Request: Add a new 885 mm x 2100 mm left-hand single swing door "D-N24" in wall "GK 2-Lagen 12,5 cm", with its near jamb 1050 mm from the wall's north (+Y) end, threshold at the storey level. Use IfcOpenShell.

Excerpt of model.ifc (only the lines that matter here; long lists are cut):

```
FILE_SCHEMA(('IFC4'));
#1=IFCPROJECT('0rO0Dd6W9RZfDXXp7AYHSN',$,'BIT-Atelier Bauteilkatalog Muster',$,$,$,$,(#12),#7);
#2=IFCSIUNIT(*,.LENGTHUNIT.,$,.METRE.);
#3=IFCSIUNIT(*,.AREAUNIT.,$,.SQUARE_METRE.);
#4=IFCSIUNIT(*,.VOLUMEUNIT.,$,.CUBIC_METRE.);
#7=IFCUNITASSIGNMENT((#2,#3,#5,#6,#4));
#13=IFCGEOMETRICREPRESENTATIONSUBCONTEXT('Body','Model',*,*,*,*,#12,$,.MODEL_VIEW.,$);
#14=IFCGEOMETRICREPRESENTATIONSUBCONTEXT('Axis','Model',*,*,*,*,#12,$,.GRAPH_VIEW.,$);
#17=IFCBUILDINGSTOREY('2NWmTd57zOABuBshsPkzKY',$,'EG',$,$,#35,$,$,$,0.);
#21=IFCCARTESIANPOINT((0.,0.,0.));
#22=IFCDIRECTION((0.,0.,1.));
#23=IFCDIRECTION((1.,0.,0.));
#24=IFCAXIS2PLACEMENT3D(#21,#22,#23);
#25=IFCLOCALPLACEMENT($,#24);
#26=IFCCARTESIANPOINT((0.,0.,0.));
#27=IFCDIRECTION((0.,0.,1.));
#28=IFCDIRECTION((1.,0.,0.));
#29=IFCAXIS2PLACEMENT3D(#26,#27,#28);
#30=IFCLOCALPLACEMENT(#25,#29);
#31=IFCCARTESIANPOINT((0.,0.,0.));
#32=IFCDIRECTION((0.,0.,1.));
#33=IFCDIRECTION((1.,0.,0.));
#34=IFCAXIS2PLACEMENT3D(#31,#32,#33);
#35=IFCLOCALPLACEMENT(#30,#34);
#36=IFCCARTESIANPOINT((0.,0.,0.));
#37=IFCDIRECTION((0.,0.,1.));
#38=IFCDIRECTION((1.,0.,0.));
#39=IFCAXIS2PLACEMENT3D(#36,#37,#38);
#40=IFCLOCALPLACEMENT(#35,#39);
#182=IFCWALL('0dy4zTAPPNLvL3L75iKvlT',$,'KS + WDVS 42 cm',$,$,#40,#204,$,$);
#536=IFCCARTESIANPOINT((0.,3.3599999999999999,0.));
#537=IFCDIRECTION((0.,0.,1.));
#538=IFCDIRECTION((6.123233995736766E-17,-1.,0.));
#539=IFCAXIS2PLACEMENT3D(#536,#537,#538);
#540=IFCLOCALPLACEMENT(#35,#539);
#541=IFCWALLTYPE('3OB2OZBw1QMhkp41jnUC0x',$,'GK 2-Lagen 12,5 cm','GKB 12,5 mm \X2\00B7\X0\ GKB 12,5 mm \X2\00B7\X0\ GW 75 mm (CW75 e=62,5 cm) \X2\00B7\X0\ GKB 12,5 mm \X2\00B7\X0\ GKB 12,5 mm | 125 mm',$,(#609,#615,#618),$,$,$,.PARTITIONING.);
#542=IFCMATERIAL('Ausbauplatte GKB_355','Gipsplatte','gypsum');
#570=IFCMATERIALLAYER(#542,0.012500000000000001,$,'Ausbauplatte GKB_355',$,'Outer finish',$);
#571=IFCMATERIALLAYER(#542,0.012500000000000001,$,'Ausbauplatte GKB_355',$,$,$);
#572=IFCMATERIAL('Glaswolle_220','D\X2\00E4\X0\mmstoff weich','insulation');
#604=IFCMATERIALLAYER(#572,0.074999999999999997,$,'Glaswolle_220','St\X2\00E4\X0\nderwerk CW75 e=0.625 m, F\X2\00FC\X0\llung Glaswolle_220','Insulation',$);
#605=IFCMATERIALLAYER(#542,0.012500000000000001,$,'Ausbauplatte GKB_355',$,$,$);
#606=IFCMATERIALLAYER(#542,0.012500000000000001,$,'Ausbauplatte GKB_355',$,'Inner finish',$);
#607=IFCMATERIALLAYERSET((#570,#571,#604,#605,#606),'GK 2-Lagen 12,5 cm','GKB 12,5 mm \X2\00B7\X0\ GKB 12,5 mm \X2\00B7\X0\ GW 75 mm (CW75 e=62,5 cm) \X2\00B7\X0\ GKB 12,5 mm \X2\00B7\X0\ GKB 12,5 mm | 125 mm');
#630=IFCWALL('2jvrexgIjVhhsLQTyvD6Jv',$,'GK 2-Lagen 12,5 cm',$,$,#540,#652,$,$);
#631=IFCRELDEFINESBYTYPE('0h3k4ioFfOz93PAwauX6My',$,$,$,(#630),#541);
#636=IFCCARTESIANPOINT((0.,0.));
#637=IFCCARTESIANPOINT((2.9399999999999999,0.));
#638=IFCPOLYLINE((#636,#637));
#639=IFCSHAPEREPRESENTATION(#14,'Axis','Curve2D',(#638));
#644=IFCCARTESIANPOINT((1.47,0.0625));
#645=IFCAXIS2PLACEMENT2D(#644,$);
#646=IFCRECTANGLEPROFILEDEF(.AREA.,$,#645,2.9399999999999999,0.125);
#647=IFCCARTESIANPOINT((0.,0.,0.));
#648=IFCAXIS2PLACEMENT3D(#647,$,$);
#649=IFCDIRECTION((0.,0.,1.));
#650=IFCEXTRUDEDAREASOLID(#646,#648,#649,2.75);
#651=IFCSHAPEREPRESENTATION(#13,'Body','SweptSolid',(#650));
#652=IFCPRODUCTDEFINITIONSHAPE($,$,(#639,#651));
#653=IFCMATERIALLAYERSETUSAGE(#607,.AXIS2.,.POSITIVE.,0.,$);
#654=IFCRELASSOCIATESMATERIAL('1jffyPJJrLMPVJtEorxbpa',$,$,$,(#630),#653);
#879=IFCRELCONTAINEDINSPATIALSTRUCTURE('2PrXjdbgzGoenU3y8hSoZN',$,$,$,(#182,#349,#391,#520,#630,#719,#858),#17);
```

```python
import numpy as np
import ifcopenshell
import ifcopenshell.api.feature
import ifcopenshell.api.geometry
import ifcopenshell.api.root
import ifcopenshell.api.spatial
import ifcopenshell.geom
import ifcopenshell.util.element
import ifcopenshell.util.placement
import ifcopenshell.util.representation
import ifcopenshell.util.shape
import ifcopenshell.util.unit

model = ifcopenshell.open("model.ifc")
unit_scale = ifcopenshell.util.unit.calculate_unit_scale(model)
settings = ifcopenshell.geom.settings()


def volume(element):
    """Net volume in cubic metres, openings subtracted."""
    shape = ifcopenshell.geom.create_shape(settings, element)
    return ifcopenshell.util.shape.get_volume(shape.geometry)


wall = model.by_guid("2jvrexgIjVhhsLQTyvD6Jv")
storey = ifcopenshell.util.element.get_container(wall, ifc_class="IfcBuildingStorey")
context = ifcopenshell.util.representation.get_context(model, "Model", "Body", "MODEL_VIEW")
before = volume(wall)

width, height, from_end, sill = 0.885, 2.1, 1.05, 0.0  # metres

# The wall runs along its own X axis, and the end named is its -X end.
wall_shape = ifcopenshell.geom.create_shape(settings, wall)
x, y, z = ifcopenshell.util.shape.get_vertices(wall_shape.geometry).T
start = x.min() + from_end
face, thickness = float(y.min()), float(y.max() - y.min())
wall_matrix = ifcopenshell.util.placement.get_local_placement(wall.ObjectPlacement)
level = ifcopenshell.util.placement.get_local_placement(storey.ObjectPlacement)[2, 3]


def in_wall(x, y):
    """Placement at x, y metres in the wall's axes, at sill height."""
    matrix = wall_matrix.copy()
    matrix[:, 3] = wall_matrix @ np.array([x / unit_scale, y / unit_scale, 0.0, 1.0])
    matrix[2, 3] = level + sill / unit_scale
    return matrix


# Opening: a box that overshoots both wall faces by 50 mm.
opening = ifcopenshell.api.root.create_entity(model, ifc_class="IfcOpeningElement", predefined_type="OPENING")
box = ifcopenshell.api.geometry.add_wall_representation(
    model, context=context, length=width, height=height, thickness=thickness + 0.1
)
ifcopenshell.api.geometry.assign_representation(model, product=opening, representation=box)
ifcopenshell.api.geometry.edit_object_placement(model, product=opening, matrix=in_wall(start, face - 0.05), is_si=False)
ifcopenshell.api.feature.add_feature(model, feature=opening, element=wall)

door = ifcopenshell.api.root.create_entity(model, ifc_class="IfcDoor", name="D-N24", predefined_type="DOOR")
door.OverallWidth, door.OverallHeight = width / unit_scale, height / unit_scale
door.OperationType = "SINGLE_SWING_LEFT"
body = ifcopenshell.api.geometry.add_door_representation(
    model,
    context=context,
    overall_width=door.OverallWidth,
    overall_height=door.OverallHeight,
    operation_type="SINGLE_SWING_LEFT",
    lining_properties={"LiningDepth": thickness / unit_scale, "ThresholdDepth": thickness / unit_scale},
)
ifcopenshell.api.geometry.assign_representation(model, product=door, representation=body)
ifcopenshell.api.spatial.assign_container(model, products=[door], relating_structure=storey)
ifcopenshell.api.feature.add_filling(model, opening=opening, element=door)

# The lining spans the wall, so the door starts at the wall face.
ifcopenshell.api.geometry.edit_object_placement(model, product=door, matrix=in_wall(start, face), is_si=False)

after = volume(wall)

print(f"wall volume {before:.3f} -> {after:.3f} m3")

model.write("model_v2.ifc")
```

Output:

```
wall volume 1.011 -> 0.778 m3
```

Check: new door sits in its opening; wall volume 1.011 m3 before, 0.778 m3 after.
